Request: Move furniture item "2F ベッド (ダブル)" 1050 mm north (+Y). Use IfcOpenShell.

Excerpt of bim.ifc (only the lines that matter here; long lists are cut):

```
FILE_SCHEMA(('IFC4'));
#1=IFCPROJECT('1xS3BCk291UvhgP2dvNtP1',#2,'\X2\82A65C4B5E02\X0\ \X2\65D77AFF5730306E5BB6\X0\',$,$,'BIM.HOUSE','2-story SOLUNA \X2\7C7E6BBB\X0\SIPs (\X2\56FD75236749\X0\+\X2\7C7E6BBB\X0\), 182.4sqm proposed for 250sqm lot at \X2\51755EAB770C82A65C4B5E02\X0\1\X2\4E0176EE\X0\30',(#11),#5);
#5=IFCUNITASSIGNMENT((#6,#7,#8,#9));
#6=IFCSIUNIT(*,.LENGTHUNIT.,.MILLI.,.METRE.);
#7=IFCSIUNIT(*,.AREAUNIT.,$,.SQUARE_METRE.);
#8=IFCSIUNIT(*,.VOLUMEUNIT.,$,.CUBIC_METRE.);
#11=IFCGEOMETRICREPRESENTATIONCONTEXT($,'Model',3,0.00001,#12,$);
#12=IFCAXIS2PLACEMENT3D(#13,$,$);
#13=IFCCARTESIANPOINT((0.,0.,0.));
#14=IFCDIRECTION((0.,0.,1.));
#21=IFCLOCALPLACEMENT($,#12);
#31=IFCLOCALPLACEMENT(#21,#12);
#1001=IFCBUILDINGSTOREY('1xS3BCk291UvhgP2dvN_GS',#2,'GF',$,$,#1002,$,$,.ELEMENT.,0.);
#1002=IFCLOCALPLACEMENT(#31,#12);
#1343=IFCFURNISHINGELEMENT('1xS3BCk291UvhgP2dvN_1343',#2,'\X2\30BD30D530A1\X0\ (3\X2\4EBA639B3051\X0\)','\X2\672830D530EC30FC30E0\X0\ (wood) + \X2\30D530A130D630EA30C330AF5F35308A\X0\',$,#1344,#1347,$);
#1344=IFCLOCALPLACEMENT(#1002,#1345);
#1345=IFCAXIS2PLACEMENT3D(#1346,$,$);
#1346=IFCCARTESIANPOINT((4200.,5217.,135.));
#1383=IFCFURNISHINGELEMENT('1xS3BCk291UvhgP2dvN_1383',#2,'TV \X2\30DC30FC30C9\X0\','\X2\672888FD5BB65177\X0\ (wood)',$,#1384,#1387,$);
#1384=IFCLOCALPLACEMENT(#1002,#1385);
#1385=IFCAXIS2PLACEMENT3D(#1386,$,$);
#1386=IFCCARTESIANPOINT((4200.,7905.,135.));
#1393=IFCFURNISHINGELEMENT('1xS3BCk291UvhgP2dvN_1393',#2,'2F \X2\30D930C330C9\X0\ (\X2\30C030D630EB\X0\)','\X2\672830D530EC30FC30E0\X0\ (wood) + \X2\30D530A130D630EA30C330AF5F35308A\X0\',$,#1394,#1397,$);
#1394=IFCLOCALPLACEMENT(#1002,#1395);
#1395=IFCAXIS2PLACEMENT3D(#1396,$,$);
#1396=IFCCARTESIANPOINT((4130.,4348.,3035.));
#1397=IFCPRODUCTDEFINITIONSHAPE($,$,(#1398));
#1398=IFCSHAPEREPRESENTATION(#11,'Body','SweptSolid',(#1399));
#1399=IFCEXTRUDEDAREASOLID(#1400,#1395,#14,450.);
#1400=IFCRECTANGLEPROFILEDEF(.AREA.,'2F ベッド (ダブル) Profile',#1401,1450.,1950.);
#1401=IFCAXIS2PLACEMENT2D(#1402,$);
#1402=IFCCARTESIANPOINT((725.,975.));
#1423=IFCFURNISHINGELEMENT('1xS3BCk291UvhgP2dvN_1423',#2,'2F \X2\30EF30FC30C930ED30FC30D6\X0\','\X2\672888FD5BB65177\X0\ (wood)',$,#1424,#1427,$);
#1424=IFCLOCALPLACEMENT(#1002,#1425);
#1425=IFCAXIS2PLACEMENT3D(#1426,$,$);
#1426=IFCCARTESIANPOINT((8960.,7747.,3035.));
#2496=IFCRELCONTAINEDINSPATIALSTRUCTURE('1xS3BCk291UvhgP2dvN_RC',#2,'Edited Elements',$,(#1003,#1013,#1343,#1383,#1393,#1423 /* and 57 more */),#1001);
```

```python
import ifcopenshell
import ifcopenshell.api.geometry
import ifcopenshell.util.placement
import ifcopenshell.util.unit

model = ifcopenshell.open("bim.ifc")
unit_scale = ifcopenshell.util.unit.calculate_unit_scale(model)

item = model.by_guid("1xS3BCk291UvhgP2dvN_1393")
matrix = ifcopenshell.util.placement.get_local_placement(item.ObjectPlacement)
matrix[1, 3] += 1.05 / unit_scale
ifcopenshell.api.geometry.edit_object_placement(model, product=item, matrix=matrix, is_si=False)

print(ifcopenshell.util.placement.get_local_placement(item.ObjectPlacement).round(3) + 0.0)

model.write("bim_v2.ifc")
```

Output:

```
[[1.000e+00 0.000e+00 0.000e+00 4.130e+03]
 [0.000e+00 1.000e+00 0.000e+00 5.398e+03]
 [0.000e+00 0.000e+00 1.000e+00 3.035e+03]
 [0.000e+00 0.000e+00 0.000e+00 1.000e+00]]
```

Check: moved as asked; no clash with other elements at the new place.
